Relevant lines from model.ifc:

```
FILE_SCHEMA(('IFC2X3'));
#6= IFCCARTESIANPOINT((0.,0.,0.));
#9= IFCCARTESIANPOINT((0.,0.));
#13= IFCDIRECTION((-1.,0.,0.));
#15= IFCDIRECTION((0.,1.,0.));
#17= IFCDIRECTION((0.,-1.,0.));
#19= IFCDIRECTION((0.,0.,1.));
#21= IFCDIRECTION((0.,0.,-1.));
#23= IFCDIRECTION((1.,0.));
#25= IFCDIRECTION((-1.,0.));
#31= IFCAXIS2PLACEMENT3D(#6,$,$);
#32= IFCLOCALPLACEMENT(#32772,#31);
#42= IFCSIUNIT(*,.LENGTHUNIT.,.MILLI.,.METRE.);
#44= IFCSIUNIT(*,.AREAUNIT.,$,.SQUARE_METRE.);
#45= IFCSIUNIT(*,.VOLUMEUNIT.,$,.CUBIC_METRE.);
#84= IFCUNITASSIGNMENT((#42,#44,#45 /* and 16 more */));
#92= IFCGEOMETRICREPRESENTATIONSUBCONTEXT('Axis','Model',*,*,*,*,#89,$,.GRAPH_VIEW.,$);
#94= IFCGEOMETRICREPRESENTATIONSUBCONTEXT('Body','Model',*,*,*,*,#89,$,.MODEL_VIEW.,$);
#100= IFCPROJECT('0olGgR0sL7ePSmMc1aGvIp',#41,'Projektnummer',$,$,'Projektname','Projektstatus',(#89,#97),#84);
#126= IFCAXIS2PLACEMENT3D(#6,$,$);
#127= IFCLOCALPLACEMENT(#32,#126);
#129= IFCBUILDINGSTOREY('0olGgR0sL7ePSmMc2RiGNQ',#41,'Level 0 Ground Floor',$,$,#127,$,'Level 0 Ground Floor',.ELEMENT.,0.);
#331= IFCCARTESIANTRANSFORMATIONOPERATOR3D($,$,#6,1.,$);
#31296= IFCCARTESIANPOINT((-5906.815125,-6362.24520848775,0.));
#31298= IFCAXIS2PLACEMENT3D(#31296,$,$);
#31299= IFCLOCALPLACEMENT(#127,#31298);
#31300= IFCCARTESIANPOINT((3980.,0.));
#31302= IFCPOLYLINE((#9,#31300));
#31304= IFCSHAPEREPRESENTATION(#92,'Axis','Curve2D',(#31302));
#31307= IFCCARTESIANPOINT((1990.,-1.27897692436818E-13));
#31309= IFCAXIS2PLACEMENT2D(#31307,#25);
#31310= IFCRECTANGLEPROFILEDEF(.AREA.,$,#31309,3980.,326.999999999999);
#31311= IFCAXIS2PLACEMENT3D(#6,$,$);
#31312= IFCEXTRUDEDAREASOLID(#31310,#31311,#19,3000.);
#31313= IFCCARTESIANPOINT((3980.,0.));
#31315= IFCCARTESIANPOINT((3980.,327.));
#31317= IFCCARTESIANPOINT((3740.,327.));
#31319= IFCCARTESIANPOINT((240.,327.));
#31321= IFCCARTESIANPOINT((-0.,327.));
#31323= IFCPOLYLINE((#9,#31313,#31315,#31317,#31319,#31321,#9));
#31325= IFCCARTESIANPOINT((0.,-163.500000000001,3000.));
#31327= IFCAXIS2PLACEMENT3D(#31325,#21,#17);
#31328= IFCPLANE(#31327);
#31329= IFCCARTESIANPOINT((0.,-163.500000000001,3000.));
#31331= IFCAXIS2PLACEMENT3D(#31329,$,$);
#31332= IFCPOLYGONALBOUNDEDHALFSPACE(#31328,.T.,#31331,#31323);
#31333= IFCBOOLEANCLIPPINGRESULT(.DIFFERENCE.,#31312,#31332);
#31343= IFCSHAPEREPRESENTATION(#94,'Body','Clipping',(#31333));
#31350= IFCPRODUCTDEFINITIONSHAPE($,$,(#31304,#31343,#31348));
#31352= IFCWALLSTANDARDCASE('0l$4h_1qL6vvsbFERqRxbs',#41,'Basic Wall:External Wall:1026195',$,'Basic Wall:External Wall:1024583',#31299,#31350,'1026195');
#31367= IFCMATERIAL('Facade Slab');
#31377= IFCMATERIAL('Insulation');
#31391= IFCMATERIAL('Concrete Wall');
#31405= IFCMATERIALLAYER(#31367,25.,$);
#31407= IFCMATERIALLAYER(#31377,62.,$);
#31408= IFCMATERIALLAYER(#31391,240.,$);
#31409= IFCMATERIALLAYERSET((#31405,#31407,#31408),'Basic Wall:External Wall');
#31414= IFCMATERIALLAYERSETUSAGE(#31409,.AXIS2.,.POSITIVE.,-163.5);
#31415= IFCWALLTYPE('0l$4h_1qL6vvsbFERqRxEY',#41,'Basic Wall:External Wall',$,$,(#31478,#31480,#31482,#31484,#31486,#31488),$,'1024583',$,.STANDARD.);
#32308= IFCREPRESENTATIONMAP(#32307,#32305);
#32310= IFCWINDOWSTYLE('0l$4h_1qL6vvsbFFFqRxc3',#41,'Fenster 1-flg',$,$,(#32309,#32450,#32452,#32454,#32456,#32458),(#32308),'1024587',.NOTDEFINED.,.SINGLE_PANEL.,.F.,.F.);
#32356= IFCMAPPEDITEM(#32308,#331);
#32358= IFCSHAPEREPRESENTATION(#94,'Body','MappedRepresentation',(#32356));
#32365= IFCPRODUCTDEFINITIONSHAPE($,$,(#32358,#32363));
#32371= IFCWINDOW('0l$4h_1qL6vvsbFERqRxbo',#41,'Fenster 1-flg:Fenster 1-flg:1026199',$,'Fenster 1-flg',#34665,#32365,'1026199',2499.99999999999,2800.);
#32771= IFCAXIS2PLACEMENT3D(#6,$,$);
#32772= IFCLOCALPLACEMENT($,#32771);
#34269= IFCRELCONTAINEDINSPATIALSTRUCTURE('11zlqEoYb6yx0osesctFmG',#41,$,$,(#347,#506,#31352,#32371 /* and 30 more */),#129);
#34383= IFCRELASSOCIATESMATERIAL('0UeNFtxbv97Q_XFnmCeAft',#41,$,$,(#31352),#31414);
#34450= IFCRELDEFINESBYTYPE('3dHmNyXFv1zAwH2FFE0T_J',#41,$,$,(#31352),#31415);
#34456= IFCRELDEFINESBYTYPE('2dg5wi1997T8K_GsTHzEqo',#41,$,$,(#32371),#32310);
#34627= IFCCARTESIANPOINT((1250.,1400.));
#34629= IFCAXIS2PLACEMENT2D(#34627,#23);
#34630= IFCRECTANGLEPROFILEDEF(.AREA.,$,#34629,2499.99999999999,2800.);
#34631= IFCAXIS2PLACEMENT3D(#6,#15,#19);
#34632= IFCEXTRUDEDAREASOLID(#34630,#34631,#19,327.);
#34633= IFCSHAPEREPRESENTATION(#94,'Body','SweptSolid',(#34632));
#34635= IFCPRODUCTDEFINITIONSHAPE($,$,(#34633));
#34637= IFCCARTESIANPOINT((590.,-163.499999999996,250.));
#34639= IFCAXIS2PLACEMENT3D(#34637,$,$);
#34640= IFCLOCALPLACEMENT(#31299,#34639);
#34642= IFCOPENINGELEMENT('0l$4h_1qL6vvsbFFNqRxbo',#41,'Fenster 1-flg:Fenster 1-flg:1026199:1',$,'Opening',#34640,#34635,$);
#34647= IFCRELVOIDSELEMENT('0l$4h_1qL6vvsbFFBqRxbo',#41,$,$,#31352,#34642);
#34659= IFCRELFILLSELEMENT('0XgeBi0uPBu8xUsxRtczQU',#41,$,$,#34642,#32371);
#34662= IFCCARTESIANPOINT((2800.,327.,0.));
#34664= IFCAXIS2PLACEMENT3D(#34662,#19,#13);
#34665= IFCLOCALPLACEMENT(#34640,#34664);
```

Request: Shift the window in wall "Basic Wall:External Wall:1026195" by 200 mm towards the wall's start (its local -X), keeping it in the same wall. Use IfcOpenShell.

```python
import ifcopenshell
import ifcopenshell.api.geometry
import ifcopenshell.util.placement

model = ifcopenshell.open("model.ifc")

window = model.by_guid("0l$4h_1qL6vvsbFERqRxbo")
opening = window.FillsVoids[0].RelatingOpeningElement
wall = opening.VoidsElements[0].RelatingBuildingElement

wall_matrix = ifcopenshell.util.placement.get_local_placement(wall.ObjectPlacement)
shift = wall_matrix[:3, 0] * -200.0
before = ifcopenshell.util.placement.get_local_placement(window.ObjectPlacement)[:3, 3].copy()

# The window is placed relative to its opening, so it follows when the opening moves.
matrix = ifcopenshell.util.placement.get_local_placement(opening.ObjectPlacement)
matrix[:3, 3] += shift
ifcopenshell.api.geometry.edit_object_placement(
    model, product=opening, matrix=matrix, is_si=False, should_transform_children=True
)

after = ifcopenshell.util.placement.get_local_placement(window.ObjectPlacement)[:3, 3]
print("window moved by", (after - before).round(3) + 0.0)

model.write("model_edited.ifc")
```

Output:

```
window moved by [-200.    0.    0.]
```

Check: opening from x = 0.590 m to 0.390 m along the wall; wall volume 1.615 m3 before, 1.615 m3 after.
